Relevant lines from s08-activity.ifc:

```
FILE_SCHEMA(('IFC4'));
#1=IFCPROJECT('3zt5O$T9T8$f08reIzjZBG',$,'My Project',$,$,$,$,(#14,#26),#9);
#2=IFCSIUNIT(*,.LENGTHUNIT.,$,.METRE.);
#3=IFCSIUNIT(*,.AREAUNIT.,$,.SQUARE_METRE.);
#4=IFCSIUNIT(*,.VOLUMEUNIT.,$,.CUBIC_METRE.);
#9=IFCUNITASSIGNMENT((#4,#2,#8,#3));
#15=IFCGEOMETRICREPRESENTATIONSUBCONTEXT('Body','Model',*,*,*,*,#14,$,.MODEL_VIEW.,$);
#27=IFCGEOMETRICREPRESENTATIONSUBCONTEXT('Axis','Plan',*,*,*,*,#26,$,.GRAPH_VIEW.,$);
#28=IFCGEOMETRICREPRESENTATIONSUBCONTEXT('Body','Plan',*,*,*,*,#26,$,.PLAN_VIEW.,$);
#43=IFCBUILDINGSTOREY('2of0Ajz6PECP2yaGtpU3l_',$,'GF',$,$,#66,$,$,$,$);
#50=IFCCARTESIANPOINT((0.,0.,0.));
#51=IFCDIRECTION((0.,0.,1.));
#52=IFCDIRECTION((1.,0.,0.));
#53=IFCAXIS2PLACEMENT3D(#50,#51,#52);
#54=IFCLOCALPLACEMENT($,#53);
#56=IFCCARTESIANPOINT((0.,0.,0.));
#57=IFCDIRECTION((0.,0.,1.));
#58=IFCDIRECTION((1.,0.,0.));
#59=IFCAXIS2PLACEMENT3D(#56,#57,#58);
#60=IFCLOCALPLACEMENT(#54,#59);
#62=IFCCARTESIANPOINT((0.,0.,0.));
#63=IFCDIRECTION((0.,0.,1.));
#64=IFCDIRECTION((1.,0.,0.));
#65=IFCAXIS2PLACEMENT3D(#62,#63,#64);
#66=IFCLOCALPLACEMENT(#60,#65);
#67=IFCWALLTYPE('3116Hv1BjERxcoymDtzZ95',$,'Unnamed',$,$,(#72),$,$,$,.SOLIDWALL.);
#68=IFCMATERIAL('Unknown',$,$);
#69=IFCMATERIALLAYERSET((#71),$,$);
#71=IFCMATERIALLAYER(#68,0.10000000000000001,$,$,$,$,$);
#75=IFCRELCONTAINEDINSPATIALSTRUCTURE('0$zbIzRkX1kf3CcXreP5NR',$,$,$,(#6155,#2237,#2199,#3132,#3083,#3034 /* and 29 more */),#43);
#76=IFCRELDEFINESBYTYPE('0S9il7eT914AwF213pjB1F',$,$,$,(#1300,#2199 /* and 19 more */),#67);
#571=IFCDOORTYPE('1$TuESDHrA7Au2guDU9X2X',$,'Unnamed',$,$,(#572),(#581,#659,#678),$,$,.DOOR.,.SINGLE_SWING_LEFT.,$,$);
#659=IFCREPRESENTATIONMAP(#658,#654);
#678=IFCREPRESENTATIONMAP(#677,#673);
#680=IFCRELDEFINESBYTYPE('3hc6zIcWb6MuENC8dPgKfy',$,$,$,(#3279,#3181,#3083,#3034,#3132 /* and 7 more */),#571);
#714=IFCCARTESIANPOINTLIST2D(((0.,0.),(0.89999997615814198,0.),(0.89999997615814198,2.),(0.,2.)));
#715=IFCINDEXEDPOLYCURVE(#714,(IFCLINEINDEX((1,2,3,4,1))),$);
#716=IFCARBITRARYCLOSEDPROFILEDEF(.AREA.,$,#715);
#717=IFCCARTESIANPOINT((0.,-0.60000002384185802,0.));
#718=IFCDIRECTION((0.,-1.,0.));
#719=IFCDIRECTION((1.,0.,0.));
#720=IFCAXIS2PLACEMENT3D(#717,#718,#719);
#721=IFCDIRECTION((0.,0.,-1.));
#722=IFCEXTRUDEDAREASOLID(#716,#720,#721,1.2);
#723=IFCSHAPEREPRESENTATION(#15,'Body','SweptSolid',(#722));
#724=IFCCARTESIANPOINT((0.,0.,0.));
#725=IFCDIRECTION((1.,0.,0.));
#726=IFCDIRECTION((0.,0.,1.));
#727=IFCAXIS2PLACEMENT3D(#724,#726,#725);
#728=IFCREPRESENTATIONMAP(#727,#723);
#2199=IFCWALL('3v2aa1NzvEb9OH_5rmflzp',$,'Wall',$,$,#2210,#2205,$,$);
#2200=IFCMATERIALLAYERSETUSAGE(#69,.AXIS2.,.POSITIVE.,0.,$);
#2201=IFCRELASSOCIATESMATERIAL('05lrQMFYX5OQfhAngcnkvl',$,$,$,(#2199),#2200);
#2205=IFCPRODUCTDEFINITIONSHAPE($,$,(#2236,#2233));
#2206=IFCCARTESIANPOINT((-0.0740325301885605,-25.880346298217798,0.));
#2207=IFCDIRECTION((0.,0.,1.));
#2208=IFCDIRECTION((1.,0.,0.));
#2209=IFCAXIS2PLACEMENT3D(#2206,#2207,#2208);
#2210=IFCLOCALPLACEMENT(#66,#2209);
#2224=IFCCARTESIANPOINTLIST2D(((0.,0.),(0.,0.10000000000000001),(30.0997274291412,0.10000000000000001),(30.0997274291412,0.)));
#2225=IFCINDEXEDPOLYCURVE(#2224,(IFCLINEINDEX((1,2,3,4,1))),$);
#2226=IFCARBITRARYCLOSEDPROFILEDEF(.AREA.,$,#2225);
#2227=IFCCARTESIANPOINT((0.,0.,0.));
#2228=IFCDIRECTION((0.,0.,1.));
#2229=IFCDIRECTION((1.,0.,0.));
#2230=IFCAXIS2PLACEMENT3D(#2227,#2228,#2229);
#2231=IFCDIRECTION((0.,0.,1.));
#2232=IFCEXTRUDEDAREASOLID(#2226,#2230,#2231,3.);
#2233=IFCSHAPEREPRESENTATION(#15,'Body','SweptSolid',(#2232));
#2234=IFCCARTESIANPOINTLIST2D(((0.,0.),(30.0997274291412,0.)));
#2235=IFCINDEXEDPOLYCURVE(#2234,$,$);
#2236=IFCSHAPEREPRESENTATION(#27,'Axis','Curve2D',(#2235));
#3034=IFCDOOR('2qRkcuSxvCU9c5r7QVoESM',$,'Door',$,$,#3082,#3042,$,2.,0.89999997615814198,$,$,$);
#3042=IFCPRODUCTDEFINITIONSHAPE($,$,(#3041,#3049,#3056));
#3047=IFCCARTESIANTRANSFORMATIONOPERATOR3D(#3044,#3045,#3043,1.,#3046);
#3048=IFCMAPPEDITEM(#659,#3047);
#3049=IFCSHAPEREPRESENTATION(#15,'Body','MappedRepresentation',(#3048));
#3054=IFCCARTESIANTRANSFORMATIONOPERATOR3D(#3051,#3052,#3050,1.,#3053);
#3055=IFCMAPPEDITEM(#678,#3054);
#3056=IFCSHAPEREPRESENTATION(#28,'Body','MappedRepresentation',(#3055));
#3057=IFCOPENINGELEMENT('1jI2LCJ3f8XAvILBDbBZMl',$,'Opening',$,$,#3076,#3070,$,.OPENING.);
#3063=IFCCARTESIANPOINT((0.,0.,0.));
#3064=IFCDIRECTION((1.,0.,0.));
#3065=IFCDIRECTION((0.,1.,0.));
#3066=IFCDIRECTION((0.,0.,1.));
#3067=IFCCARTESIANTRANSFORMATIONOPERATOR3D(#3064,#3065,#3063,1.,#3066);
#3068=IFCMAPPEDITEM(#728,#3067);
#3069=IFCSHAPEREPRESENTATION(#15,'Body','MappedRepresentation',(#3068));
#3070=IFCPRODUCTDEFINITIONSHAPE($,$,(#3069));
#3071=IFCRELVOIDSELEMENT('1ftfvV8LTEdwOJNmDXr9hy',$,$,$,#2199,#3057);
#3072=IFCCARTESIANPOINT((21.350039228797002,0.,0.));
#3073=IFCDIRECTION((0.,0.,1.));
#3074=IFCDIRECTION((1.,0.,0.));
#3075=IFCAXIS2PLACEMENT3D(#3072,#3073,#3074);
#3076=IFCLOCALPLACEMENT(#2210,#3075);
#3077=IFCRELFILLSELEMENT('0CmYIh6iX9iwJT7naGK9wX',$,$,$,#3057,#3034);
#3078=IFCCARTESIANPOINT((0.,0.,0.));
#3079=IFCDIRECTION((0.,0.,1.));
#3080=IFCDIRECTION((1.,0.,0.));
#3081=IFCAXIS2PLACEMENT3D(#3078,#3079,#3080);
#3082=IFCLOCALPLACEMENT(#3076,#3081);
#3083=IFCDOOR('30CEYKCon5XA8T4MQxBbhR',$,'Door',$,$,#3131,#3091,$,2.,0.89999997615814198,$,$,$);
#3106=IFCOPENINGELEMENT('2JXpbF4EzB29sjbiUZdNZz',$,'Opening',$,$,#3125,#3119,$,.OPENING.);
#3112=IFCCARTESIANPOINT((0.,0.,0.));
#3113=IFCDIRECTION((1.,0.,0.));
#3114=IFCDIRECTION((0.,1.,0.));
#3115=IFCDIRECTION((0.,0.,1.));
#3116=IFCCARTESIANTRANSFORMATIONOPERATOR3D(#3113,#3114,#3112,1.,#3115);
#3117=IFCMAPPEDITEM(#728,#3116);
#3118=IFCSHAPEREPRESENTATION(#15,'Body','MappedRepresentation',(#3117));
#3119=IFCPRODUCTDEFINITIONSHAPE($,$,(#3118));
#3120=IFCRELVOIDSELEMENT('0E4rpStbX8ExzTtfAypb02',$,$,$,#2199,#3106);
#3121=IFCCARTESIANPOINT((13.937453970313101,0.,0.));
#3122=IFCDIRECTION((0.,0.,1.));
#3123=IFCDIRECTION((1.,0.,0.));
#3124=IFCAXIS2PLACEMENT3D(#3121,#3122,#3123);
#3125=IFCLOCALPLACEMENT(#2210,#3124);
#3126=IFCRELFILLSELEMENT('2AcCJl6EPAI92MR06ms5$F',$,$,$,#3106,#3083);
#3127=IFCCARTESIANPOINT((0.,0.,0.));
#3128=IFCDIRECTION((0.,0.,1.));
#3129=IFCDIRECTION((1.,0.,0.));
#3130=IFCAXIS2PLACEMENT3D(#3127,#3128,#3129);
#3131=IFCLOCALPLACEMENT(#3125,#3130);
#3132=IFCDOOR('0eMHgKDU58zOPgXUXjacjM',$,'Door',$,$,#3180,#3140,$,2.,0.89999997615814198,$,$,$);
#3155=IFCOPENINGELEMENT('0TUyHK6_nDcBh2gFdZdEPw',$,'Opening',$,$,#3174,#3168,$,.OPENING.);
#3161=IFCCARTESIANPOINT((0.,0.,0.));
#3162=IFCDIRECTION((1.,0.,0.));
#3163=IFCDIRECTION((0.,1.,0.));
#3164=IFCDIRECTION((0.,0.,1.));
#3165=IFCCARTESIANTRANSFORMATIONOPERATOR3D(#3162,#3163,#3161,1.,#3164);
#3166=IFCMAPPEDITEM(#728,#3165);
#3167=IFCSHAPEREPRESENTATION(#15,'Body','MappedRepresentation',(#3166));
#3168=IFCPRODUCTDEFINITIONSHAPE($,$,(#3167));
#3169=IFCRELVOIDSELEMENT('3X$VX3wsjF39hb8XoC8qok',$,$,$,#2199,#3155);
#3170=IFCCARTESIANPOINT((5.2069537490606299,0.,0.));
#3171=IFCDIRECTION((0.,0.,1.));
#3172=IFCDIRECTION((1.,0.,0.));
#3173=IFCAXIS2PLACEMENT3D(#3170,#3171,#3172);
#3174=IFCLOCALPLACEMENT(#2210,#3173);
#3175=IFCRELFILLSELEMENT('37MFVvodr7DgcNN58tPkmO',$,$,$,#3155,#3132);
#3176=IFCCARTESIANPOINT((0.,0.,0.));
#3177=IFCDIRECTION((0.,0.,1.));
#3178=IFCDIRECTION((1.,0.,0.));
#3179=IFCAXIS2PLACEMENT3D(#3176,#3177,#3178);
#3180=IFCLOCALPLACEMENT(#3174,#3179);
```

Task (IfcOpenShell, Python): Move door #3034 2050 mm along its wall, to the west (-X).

```python
import ifcopenshell
import ifcopenshell.api.geometry
import ifcopenshell.util.placement

model = ifcopenshell.open("s08-activity.ifc")

door = model.by_guid("2qRkcuSxvCU9c5r7QVoESM")
opening = door.FillsVoids[0].RelatingOpeningElement
wall = opening.VoidsElements[0].RelatingBuildingElement

wall_matrix = ifcopenshell.util.placement.get_local_placement(wall.ObjectPlacement)
shift = wall_matrix[:3, 0] * -2.05
before = ifcopenshell.util.placement.get_local_placement(door.ObjectPlacement)[:3, 3].copy()

# The door is placed relative to its opening, so it follows when the opening moves.
matrix = ifcopenshell.util.placement.get_local_placement(opening.ObjectPlacement)
matrix[:3, 3] += shift
ifcopenshell.api.geometry.edit_object_placement(
    model, product=opening, matrix=matrix, is_si=False, should_transform_children=True
)

after = ifcopenshell.util.placement.get_local_placement(door.ObjectPlacement)[:3, 3]
print("door moved by", (after - before).round(3) + 0.0)

model.write("s08-activity_updated.ifc")
```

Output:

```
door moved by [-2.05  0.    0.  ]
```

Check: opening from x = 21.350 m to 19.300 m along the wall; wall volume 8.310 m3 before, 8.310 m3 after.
